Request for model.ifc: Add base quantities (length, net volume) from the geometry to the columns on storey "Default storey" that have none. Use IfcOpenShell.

First a look at what the model holds.

```python
import ifcopenshell
import ifcopenshell.util.element
import ifcopenshell.util.unit

model = ifcopenshell.open("model.ifc")
print(model.schema)
for unit_type in ("LENGTHUNIT", "AREAUNIT", "VOLUMEUNIT"):
    print(unit_type, ifcopenshell.util.unit.calculate_unit_scale(model, unit_type))
storey = next(s for s in model.by_type("IfcBuildingStorey") if s.Name == "Default storey")
columns = [e for e in ifcopenshell.util.element.get_decomposition(storey) if e.is_a("IfcColumn")]
for e in sorted(columns, key=lambda e: e.id()):
    print(e.id(), e.is_a(), e.Name, list(ifcopenshell.util.element.get_psets(e, qtos_only=True)), sep=" | ")
```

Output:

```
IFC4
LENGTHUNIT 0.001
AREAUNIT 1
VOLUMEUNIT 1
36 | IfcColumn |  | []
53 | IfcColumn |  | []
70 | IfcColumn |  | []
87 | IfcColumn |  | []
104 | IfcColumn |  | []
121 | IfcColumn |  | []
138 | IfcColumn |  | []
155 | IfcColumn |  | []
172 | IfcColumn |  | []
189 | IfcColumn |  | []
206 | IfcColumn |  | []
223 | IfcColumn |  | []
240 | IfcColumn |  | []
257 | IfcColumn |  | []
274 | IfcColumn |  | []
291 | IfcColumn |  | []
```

```python
import ifcopenshell
import ifcopenshell.api.pset
import ifcopenshell.geom
import ifcopenshell.util.element
import ifcopenshell.util.shape
import ifcopenshell.util.unit

model = ifcopenshell.open("model.ifc")
unit_scale = ifcopenshell.util.unit.calculate_unit_scale(model)
volume_scale = ifcopenshell.util.unit.calculate_unit_scale(model, "VOLUMEUNIT")
settings = ifcopenshell.geom.settings()

storey = next(s for s in model.by_type("IfcBuildingStorey") if s.Name == "Default storey")
columns = [e for e in ifcopenshell.util.element.get_decomposition(storey) if e.is_a("IfcColumn")]

for e in sorted(columns, key=lambda e: e.id()):
    if ifcopenshell.util.element.get_psets(e, qtos_only=True, should_inherit=False):
        continue
    # Geometry comes back in metres, in the element's own axes.
    shape = ifcopenshell.geom.create_shape(settings, e)
    values = {
        "Length": ifcopenshell.util.shape.get_z(shape.geometry) / unit_scale,
        "NetVolume": ifcopenshell.util.shape.get_volume(shape.geometry) / volume_scale,
    }
    qto = ifcopenshell.api.pset.add_qto(model, product=e, name="Qto_ColumnBaseQuantities")
    ifcopenshell.api.pset.edit_qto(model, qto=qto, properties=values)
    print(e.id(), {k: round(v, 3) for k, v in values.items()})

model.write("model_rev.ifc")
```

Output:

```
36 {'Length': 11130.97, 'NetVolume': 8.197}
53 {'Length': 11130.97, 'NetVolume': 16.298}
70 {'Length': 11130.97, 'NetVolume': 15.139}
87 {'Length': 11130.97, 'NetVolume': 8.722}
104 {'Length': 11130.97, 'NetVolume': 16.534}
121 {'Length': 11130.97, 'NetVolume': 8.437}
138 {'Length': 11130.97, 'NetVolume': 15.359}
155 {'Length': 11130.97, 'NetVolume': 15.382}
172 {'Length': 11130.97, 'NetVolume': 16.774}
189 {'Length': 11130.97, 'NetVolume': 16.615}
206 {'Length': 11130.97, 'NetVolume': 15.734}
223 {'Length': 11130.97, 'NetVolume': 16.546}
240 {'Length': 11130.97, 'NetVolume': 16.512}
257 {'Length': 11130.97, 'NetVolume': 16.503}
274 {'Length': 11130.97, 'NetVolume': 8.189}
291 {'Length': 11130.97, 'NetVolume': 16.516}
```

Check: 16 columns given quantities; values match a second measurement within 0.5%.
